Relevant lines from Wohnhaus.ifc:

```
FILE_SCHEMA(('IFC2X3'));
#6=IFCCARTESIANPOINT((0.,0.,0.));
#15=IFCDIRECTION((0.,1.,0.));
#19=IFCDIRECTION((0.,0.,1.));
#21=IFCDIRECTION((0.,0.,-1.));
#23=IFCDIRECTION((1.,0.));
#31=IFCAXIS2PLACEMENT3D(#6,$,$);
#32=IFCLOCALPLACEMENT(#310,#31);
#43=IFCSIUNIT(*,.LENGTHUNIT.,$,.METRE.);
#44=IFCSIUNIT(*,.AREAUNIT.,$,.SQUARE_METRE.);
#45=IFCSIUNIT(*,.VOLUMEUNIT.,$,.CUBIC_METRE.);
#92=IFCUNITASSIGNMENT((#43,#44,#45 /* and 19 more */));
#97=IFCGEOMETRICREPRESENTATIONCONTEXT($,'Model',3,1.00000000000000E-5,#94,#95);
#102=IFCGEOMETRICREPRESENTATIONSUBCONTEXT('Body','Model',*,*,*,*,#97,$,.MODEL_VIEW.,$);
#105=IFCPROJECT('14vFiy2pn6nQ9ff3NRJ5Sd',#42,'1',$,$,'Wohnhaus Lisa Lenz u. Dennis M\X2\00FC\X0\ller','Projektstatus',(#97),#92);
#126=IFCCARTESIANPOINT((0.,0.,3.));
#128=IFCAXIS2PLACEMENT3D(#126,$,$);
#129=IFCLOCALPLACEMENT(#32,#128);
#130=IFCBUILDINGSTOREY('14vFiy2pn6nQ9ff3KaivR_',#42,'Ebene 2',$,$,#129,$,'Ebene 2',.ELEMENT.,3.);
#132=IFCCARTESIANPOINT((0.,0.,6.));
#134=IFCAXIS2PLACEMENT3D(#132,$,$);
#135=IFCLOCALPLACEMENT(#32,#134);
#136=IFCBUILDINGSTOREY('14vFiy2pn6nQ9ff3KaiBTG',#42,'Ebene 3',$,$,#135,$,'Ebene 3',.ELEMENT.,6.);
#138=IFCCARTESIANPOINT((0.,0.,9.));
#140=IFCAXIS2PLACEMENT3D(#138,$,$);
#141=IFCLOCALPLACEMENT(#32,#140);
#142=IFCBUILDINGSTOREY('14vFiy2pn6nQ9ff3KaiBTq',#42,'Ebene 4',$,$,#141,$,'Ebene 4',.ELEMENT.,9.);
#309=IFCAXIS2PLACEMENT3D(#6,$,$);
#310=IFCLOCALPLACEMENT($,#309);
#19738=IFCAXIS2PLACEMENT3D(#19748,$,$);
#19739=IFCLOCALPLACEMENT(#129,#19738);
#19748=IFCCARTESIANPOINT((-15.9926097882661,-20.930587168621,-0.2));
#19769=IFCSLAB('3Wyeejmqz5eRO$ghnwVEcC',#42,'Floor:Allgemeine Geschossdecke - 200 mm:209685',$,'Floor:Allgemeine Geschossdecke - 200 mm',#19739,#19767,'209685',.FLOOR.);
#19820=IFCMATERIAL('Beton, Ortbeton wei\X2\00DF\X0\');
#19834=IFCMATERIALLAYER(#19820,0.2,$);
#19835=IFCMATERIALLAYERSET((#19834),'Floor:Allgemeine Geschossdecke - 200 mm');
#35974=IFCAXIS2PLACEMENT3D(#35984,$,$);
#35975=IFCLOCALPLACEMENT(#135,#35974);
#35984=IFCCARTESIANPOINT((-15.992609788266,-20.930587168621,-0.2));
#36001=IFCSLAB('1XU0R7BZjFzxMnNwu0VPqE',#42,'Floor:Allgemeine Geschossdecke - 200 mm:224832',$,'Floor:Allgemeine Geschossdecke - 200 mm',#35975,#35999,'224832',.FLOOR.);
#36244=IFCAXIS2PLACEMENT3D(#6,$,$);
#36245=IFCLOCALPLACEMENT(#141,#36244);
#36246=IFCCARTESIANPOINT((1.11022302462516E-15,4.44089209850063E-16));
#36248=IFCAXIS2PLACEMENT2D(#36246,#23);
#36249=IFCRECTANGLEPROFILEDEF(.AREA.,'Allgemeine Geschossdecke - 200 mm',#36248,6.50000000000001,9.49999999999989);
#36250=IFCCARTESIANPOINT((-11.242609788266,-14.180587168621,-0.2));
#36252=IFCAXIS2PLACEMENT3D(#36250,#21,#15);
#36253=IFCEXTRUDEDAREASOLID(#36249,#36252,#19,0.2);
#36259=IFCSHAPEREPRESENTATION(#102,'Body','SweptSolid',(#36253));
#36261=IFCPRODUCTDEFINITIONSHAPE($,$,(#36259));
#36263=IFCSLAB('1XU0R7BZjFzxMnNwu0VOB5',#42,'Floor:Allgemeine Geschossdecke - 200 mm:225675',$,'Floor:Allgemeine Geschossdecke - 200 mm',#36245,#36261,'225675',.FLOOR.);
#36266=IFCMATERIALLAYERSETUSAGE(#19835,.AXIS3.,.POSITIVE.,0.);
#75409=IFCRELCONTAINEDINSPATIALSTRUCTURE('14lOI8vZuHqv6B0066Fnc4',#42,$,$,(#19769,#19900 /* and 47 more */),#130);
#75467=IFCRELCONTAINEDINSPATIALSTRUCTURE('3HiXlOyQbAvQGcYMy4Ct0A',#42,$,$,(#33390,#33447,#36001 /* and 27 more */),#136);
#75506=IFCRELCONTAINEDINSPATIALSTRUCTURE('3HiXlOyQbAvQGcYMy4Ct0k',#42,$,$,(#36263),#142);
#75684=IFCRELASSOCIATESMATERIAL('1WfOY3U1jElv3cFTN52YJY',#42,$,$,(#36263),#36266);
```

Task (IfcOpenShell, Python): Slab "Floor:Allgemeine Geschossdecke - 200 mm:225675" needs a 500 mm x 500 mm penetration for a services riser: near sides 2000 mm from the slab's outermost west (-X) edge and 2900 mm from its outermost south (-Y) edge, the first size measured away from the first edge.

```python
import numpy as np
import ifcopenshell
import ifcopenshell.api.feature
import ifcopenshell.api.geometry
import ifcopenshell.api.root
import ifcopenshell.geom
import ifcopenshell.util.placement
import ifcopenshell.util.representation
import ifcopenshell.util.shape
import ifcopenshell.util.unit

model = ifcopenshell.open("Wohnhaus.ifc")
unit_scale = ifcopenshell.util.unit.calculate_unit_scale(model)
settings = ifcopenshell.geom.settings()


def volume(element):
    """Net volume in cubic metres, openings subtracted."""
    shape = ifcopenshell.geom.create_shape(settings, element)
    return ifcopenshell.util.shape.get_volume(shape.geometry)


slab = model.by_id(36263)
before = volume(slab)

# Extent in the slab's own axes, in metres. The edges named are its -X and -Y sides.
slab_shape = ifcopenshell.geom.create_shape(settings, slab)
vertices = ifcopenshell.util.shape.get_vertices(slab_shape.geometry)
x_min, y_min, bottom = vertices.min(axis=0)
top = vertices[:, 2].max()

opening = ifcopenshell.api.root.create_entity(model, ifc_class="IfcOpeningElement", name="Services riser opening")
context = ifcopenshell.util.representation.get_context(model, "Model", "Body", "MODEL_VIEW")
width, depth = 0.5, 0.5
outline = [(0.0, 0.0), (width, 0.0), (width, depth), (0.0, depth), (0.0, 0.0)]
# Overshoot both faces by 50 mm so the cut is clean.
shape = ifcopenshell.api.geometry.add_slab_representation(
    model, context=context, depth=top - bottom + 0.1, polyline=outline
)
ifcopenshell.api.geometry.assign_representation(model, product=opening, representation=shape)

matrix = ifcopenshell.util.placement.get_local_placement(slab.ObjectPlacement)
matrix[:, 3] = matrix @ np.append(np.array([x_min + 2, y_min + 2.9, bottom - 0.05]) / unit_scale, 1.0)
ifcopenshell.api.geometry.edit_object_placement(model, product=opening, matrix=matrix, is_si=False)
ifcopenshell.api.feature.add_feature(model, feature=opening, element=slab)

after = volume(slab)

print(f"slab volume {before:.3f} -> {after:.3f} m3")

model.write("Wohnhaus-out.ifc")
```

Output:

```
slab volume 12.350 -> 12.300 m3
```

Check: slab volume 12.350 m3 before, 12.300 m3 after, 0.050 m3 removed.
